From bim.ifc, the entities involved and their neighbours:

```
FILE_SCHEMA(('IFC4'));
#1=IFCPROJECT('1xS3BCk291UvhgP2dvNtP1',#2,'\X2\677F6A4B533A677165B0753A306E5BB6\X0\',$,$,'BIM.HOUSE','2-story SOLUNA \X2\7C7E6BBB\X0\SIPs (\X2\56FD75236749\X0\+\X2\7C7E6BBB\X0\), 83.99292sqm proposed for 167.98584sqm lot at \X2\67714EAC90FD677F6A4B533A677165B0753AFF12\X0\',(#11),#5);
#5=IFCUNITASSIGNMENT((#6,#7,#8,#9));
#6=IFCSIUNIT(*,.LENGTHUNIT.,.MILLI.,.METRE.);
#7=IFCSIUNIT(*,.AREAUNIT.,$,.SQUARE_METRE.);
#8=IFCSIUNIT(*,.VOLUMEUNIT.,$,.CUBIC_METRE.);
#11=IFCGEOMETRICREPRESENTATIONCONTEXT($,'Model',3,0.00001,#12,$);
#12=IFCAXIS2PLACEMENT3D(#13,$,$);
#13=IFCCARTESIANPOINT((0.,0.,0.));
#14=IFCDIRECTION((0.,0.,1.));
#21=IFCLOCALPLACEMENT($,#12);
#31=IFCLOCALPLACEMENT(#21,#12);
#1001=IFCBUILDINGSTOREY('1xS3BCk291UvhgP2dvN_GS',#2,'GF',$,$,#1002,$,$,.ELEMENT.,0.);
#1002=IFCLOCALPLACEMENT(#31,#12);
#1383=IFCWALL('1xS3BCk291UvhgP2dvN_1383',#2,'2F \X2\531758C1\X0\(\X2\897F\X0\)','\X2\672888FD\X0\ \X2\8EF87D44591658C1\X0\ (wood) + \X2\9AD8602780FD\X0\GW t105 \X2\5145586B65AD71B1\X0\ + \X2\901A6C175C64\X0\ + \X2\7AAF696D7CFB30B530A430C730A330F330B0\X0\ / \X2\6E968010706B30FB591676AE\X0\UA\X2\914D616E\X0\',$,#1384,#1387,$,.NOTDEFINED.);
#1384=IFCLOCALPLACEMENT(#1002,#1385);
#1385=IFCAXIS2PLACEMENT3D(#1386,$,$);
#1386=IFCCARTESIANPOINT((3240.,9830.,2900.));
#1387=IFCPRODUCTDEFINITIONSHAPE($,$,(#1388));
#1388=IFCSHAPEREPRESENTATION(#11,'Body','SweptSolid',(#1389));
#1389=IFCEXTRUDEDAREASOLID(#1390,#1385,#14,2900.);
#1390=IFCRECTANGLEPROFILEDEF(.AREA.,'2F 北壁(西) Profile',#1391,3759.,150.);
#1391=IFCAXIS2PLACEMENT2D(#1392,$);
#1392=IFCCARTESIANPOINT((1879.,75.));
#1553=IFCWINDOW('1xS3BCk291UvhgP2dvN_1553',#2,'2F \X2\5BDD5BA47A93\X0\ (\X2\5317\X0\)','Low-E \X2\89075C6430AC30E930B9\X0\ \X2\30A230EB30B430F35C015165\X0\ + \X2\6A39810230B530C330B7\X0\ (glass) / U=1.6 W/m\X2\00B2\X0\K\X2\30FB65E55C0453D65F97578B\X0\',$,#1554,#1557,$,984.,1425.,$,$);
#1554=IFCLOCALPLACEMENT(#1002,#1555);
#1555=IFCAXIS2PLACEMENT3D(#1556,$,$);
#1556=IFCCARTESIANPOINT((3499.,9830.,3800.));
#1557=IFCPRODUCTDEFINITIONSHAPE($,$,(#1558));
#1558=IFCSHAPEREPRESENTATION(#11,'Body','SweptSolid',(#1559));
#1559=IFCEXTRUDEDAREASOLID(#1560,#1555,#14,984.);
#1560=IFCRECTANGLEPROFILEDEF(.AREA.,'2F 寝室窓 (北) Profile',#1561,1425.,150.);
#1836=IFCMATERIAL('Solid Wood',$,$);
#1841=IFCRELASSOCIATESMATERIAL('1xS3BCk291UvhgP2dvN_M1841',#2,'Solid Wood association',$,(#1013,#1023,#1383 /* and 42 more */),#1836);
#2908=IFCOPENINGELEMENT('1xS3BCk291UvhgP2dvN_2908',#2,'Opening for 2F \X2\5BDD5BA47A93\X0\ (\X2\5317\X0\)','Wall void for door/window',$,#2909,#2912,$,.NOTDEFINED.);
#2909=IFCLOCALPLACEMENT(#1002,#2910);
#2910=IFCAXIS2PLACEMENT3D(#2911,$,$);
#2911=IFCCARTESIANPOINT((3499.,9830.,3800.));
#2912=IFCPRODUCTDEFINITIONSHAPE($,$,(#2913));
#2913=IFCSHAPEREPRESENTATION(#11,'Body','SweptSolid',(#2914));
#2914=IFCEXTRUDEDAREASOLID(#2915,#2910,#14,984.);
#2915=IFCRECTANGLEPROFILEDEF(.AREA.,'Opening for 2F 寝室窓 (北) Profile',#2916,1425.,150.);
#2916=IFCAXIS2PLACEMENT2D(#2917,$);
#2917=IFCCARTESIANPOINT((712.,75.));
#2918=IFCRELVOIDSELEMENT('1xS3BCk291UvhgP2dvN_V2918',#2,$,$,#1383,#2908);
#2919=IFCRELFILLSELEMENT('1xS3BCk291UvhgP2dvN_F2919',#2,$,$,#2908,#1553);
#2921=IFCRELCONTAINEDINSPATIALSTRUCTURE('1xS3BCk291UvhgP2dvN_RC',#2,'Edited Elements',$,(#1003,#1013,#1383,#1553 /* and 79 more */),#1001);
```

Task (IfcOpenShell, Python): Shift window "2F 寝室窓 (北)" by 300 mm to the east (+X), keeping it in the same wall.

```python
import ifcopenshell
import ifcopenshell.api.geometry
import ifcopenshell.util.placement

model = ifcopenshell.open("bim.ifc")

window = model.by_guid("1xS3BCk291UvhgP2dvN_1553")
opening = window.FillsVoids[0].RelatingOpeningElement
wall = opening.VoidsElements[0].RelatingBuildingElement

wall_matrix = ifcopenshell.util.placement.get_local_placement(wall.ObjectPlacement)
shift = wall_matrix[:3, 0] * 300.0
before = ifcopenshell.util.placement.get_local_placement(window.ObjectPlacement)[:3, 3].copy()

# The window is not placed relative to its opening, so move both.
for product in (opening, window):
    matrix = ifcopenshell.util.placement.get_local_placement(product.ObjectPlacement)
    matrix[:3, 3] += shift
    ifcopenshell.api.geometry.edit_object_placement(model, product=product, matrix=matrix, is_si=False)

after = ifcopenshell.util.placement.get_local_placement(window.ObjectPlacement)[:3, 3]
print("window moved by", (after - before).round(3) + 0.0)

model.write("bim-out.ifc")
```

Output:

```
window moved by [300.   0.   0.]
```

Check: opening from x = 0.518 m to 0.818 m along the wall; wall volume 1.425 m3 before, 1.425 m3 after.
